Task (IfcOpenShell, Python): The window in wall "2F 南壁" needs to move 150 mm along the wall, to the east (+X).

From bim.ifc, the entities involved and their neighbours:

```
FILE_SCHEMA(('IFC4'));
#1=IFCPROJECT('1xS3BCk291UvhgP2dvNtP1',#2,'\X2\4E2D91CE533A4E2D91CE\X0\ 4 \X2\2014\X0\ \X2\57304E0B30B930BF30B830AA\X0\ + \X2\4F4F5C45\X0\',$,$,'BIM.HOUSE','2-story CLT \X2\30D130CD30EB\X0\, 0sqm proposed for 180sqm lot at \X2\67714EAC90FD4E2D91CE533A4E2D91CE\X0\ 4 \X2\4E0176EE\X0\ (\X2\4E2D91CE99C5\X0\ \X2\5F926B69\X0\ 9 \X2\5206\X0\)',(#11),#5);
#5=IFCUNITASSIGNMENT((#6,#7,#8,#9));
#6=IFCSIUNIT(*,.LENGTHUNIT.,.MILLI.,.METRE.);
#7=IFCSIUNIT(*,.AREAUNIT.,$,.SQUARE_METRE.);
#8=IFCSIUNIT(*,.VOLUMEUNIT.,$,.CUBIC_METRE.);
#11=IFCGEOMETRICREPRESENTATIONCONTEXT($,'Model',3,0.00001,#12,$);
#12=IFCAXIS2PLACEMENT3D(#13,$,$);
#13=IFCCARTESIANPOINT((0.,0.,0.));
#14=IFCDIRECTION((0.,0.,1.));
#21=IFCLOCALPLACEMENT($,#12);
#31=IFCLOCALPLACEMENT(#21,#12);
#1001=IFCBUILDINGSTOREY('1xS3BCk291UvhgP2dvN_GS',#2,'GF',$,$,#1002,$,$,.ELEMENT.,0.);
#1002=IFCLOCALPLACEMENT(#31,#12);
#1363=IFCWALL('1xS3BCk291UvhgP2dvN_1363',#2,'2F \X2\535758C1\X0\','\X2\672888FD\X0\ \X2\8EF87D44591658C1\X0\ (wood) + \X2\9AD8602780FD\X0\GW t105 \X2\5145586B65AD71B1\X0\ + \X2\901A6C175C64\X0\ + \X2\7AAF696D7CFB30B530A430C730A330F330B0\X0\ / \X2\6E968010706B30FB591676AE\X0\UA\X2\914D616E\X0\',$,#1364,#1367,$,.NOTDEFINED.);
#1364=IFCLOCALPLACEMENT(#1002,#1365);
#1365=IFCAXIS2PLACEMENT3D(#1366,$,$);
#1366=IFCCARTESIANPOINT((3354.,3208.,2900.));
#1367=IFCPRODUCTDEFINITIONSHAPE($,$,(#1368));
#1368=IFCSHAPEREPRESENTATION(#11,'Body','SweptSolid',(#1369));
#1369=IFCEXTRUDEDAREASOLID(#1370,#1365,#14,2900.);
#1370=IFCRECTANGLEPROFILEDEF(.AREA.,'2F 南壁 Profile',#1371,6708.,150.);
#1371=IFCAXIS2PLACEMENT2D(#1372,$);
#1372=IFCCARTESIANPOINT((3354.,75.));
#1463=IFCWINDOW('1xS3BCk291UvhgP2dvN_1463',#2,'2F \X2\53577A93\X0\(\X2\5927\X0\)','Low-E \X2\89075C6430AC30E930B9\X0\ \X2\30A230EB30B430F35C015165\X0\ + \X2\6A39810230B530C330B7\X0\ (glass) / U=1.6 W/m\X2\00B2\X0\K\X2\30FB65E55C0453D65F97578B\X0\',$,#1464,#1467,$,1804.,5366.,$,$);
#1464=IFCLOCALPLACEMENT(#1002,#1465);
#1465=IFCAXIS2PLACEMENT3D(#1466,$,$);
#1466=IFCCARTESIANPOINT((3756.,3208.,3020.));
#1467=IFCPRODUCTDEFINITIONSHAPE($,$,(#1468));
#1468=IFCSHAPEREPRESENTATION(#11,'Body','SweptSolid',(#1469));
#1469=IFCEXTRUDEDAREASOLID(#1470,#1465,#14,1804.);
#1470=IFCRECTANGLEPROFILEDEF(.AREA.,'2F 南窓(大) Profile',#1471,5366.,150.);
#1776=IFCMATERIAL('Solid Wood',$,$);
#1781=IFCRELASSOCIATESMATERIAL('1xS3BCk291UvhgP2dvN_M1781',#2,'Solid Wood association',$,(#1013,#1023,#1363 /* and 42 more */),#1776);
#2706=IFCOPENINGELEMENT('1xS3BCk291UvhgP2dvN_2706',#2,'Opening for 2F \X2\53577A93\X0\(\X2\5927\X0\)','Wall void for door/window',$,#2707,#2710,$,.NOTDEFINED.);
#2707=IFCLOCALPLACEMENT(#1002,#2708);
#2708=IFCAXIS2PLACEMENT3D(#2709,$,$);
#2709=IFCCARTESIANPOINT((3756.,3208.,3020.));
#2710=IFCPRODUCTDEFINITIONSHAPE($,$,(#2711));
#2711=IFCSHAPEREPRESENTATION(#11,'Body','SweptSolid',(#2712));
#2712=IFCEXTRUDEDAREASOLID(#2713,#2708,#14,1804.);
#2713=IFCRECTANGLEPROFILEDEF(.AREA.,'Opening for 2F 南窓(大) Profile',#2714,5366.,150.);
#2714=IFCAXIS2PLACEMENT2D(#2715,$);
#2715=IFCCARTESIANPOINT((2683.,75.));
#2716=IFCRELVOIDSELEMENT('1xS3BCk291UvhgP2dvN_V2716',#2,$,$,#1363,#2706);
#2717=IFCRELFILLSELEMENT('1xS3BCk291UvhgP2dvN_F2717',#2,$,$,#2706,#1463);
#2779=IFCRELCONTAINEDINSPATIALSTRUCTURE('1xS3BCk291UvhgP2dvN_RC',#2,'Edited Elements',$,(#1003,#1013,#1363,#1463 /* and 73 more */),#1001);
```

```python
import ifcopenshell
import ifcopenshell.api.geometry
import ifcopenshell.util.placement
import ifcopenshell.util.unit

model = ifcopenshell.open("bim.ifc")
unit_scale = ifcopenshell.util.unit.calculate_unit_scale(model)

window = model.by_guid("1xS3BCk291UvhgP2dvN_1463")
opening = window.FillsVoids[0].RelatingOpeningElement
wall = opening.VoidsElements[0].RelatingBuildingElement

wall_matrix = ifcopenshell.util.placement.get_local_placement(wall.ObjectPlacement)
shift = wall_matrix[:3, 0] * 0.15 / unit_scale
before = ifcopenshell.util.placement.get_local_placement(window.ObjectPlacement)[:3, 3].copy()

# The window is not placed relative to its opening, so move both.
for product in (opening, window):
    matrix = ifcopenshell.util.placement.get_local_placement(product.ObjectPlacement)
    matrix[:3, 3] += shift
    ifcopenshell.api.geometry.edit_object_placement(model, product=product, matrix=matrix, is_si=False)

after = ifcopenshell.util.placement.get_local_placement(window.ObjectPlacement)[:3, 3]
print("window moved by", (after - before).round(3) + 0.0)

model.write("bim_rev.ifc")
```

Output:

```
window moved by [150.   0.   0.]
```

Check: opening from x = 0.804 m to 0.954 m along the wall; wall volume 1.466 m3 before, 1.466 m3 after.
